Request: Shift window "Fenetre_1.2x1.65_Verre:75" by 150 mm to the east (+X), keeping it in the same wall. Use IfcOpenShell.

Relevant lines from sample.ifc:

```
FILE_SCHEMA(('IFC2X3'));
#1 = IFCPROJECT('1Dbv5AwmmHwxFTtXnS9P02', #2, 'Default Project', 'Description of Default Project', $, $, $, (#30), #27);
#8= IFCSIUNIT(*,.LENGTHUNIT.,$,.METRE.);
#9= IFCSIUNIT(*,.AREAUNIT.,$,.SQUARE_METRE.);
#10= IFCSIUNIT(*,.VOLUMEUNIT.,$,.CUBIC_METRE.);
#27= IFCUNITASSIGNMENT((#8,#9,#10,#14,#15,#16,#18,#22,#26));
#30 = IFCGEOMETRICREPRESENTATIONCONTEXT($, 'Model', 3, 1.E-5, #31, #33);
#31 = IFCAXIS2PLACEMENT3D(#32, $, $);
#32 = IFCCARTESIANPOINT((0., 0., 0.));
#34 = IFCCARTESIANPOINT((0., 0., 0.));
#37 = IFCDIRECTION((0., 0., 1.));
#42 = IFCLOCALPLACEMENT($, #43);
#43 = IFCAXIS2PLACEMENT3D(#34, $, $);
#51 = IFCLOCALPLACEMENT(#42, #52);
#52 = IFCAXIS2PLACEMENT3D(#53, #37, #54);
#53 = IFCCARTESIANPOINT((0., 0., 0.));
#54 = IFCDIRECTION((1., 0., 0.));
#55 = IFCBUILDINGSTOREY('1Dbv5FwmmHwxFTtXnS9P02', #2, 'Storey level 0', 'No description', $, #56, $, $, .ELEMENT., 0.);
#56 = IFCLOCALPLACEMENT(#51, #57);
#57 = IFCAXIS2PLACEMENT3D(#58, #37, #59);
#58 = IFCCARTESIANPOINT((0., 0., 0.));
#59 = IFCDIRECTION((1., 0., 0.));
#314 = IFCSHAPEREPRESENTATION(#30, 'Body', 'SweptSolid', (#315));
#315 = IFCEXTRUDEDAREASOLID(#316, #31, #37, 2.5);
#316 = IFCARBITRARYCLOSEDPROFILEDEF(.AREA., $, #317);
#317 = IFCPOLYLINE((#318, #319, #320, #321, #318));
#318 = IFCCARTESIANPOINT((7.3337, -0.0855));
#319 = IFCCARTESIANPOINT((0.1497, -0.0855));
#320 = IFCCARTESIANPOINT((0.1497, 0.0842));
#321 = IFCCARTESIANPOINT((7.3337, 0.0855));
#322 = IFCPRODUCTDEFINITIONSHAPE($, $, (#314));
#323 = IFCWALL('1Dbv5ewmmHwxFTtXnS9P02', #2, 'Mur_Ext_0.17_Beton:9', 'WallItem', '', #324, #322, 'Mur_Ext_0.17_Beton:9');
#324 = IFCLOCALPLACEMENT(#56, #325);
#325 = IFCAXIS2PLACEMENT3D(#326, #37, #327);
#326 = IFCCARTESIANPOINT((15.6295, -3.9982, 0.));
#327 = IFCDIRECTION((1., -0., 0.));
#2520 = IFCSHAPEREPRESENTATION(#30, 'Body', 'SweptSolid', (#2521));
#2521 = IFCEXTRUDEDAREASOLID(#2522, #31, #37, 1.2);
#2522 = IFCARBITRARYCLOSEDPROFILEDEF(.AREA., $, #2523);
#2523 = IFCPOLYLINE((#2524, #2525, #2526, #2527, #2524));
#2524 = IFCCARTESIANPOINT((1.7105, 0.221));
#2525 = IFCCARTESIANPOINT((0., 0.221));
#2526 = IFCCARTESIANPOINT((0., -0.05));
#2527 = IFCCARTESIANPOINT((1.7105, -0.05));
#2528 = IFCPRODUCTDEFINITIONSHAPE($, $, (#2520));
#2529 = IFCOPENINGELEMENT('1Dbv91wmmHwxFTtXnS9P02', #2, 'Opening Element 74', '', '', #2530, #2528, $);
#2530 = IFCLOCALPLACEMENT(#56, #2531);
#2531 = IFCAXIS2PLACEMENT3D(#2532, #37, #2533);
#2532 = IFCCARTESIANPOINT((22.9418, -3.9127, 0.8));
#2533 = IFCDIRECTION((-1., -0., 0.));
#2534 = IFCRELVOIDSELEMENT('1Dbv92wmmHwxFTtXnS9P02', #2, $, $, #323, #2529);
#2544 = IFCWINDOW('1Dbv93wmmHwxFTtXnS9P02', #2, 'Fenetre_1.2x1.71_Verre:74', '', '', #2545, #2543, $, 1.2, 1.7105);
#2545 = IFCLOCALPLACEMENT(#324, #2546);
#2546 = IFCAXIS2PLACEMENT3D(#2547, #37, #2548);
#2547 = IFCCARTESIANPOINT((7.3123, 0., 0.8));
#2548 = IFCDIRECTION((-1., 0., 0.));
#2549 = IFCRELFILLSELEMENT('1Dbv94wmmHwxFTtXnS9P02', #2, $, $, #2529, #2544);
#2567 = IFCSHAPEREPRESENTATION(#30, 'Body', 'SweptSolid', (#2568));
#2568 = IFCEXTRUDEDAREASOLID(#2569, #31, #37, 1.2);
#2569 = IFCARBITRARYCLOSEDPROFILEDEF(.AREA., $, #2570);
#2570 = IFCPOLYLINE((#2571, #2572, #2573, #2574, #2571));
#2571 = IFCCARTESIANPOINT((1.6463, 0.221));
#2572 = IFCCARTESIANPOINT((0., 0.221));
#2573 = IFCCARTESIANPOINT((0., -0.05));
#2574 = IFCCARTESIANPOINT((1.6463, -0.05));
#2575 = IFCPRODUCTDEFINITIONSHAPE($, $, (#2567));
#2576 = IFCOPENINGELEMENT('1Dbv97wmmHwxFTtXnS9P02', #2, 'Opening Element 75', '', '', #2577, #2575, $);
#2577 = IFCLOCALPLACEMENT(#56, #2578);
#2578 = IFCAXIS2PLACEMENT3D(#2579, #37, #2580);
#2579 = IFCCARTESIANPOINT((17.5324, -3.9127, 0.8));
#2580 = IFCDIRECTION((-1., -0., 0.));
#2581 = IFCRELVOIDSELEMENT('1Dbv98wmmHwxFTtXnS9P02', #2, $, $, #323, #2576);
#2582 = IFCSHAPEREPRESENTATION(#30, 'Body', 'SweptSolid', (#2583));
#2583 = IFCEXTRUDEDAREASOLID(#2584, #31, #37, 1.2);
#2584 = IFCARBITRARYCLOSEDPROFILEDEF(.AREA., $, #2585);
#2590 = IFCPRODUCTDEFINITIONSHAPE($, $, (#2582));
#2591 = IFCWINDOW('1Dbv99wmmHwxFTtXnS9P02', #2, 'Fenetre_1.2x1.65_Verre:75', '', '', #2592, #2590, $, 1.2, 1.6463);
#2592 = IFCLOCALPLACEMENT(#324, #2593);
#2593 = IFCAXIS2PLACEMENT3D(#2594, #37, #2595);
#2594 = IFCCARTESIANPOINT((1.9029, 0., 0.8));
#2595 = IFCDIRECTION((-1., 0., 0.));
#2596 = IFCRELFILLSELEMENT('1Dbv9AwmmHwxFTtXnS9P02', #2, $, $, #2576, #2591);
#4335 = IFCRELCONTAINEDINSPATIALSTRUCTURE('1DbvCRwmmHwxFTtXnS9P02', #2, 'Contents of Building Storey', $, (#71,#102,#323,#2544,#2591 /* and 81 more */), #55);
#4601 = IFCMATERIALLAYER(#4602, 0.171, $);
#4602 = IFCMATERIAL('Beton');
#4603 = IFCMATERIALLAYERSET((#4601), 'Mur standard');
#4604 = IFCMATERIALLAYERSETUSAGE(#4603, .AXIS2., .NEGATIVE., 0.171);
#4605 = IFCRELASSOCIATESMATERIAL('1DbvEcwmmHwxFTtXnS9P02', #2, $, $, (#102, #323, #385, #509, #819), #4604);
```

```python
import ifcopenshell
import ifcopenshell.api.geometry
import ifcopenshell.util.placement
import ifcopenshell.util.unit

model = ifcopenshell.open("sample.ifc")
unit_scale = ifcopenshell.util.unit.calculate_unit_scale(model)

window = model.by_guid("1Dbv99wmmHwxFTtXnS9P02")
opening = window.FillsVoids[0].RelatingOpeningElement
wall = opening.VoidsElements[0].RelatingBuildingElement

wall_matrix = ifcopenshell.util.placement.get_local_placement(wall.ObjectPlacement)
shift = wall_matrix[:3, 0] * 0.15 / unit_scale
before = ifcopenshell.util.placement.get_local_placement(window.ObjectPlacement)[:3, 3].copy()

# The window is not placed relative to its opening, so move both.
for product in (opening, window):
    matrix = ifcopenshell.util.placement.get_local_placement(product.ObjectPlacement)
    matrix[:3, 3] += shift
    ifcopenshell.api.geometry.edit_object_placement(model, product=product, matrix=matrix, is_si=False)

after = ifcopenshell.util.placement.get_local_placement(window.ObjectPlacement)[:3, 3]
print("window moved by", (after - before).round(3) + 0.0)

model.write("sample_updated.ifc")
```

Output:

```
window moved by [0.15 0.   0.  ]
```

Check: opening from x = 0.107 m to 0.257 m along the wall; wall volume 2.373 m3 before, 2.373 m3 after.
